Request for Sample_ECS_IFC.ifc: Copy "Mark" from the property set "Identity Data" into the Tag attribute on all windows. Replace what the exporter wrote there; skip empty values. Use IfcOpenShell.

First a look at what the model holds.

```python
import ifcopenshell
import ifcopenshell.util.element

model = ifcopenshell.open("Sample_ECS_IFC.ifc")
print(model.schema)
windows = model.by_type("IfcWindow")
print(len(windows), "windows")
for e in windows[:8]:
    source = ifcopenshell.util.element.get_pset(e, "Identity Data", "Mark")
    target = e.Tag
    print(e.id(), repr(source), repr(target), sep=" | ")
```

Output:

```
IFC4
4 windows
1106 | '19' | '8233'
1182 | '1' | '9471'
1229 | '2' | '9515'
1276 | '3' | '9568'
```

```python
import ifcopenshell
import ifcopenshell.util.element

model = ifcopenshell.open("Sample_ECS_IFC.ifc")

count = 0
for e in model.by_type("IfcWindow"):
    value = ifcopenshell.util.element.get_pset(e, "Identity Data", "Mark")
    current = e.Tag
    if not value or not value.strip() or current == value:
        continue
    e.Tag = value
    count += 1

print(count, "windows updated")

model.write("Sample_ECS_IFC-out.ifc")
```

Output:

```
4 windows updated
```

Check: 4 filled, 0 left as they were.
